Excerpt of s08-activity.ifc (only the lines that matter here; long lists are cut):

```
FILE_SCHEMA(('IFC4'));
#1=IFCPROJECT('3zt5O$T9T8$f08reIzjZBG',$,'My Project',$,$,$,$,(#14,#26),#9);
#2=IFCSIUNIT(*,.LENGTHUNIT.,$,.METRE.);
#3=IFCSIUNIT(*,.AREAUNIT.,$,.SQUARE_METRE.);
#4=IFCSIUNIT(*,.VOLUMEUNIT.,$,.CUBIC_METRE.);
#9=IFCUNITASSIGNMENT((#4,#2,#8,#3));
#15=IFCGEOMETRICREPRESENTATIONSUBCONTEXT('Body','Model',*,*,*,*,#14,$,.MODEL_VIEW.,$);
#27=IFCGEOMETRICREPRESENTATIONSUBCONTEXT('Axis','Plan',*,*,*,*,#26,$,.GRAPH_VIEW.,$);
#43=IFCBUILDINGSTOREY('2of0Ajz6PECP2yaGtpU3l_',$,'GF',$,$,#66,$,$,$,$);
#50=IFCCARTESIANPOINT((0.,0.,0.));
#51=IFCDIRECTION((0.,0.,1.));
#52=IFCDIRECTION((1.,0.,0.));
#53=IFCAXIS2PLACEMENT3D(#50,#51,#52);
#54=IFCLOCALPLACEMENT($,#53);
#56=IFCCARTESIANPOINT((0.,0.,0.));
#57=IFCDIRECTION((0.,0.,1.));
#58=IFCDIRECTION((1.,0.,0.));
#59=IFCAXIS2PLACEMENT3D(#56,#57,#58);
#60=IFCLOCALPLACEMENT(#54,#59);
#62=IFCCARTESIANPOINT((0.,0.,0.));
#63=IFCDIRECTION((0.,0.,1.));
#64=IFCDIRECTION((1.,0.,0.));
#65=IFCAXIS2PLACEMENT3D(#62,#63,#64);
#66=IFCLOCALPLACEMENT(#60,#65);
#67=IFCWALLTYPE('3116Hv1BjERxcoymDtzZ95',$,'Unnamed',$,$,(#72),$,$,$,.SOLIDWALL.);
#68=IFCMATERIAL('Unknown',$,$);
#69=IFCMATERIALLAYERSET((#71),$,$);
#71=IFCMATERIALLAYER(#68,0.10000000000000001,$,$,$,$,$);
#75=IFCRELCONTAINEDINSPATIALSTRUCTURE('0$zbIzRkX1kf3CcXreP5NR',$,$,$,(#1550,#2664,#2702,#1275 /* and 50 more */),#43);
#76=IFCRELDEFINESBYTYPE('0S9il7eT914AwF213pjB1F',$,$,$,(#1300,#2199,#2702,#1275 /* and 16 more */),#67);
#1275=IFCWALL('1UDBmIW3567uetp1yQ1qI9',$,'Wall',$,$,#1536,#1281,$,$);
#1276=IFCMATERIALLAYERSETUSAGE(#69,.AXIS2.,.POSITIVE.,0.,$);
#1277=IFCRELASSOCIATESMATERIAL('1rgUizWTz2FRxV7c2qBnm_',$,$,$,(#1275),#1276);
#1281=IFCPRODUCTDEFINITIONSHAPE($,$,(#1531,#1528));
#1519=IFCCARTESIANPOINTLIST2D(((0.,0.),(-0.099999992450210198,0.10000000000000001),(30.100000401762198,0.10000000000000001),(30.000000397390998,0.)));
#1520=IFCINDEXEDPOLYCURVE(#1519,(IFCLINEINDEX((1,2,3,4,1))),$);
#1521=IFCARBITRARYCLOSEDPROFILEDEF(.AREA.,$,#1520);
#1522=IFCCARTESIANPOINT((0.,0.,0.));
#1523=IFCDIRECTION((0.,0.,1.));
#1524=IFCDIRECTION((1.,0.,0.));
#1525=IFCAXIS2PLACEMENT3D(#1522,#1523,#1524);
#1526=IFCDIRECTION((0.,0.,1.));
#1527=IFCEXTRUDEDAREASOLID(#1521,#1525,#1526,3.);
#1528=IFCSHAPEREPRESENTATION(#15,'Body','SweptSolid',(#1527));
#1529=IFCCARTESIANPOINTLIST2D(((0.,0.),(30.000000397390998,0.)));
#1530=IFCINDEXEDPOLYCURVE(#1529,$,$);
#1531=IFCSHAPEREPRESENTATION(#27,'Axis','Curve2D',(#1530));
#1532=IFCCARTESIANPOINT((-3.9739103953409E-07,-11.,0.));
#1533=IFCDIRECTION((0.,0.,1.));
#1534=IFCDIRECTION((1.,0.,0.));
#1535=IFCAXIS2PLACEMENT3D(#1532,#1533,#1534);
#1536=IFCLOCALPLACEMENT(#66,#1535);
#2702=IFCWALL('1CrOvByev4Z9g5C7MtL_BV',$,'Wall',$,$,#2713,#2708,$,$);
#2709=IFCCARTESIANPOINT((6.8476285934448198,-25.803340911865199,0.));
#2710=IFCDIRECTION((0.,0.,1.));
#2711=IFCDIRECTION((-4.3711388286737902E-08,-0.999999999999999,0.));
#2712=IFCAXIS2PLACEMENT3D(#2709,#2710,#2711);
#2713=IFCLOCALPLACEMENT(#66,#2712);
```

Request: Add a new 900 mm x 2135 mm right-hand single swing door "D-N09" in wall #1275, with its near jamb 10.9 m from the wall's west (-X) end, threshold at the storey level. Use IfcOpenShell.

```python
import numpy as np
import ifcopenshell
import ifcopenshell.api.feature
import ifcopenshell.api.geometry
import ifcopenshell.api.root
import ifcopenshell.api.spatial
import ifcopenshell.geom
import ifcopenshell.util.element
import ifcopenshell.util.placement
import ifcopenshell.util.representation
import ifcopenshell.util.shape
import ifcopenshell.util.unit

model = ifcopenshell.open("s08-activity.ifc")
unit_scale = ifcopenshell.util.unit.calculate_unit_scale(model)
settings = ifcopenshell.geom.settings()


def volume(element):
    """Net volume in cubic metres, openings subtracted."""
    shape = ifcopenshell.geom.create_shape(settings, element)
    return ifcopenshell.util.shape.get_volume(shape.geometry)


wall = model.by_guid("1UDBmIW3567uetp1yQ1qI9")
storey = ifcopenshell.util.element.get_container(wall, ifc_class="IfcBuildingStorey")
context = ifcopenshell.util.representation.get_context(model, "Model", "Body", "MODEL_VIEW")
before = volume(wall)

width, height, from_end, sill = 0.9, 2.135, 10.9, 0.0  # metres

# The wall runs along its own X axis, and the end named is its -X end.
wall_shape = ifcopenshell.geom.create_shape(settings, wall)
x, y, z = ifcopenshell.util.shape.get_vertices(wall_shape.geometry).T
start = x.min() + from_end
face, thickness = float(y.min()), float(y.max() - y.min())
wall_matrix = ifcopenshell.util.placement.get_local_placement(wall.ObjectPlacement)
level = ifcopenshell.util.placement.get_local_placement(storey.ObjectPlacement)[2, 3]


def in_wall(x, y):
    """Placement at x, y metres in the wall's axes, at sill height."""
    matrix = wall_matrix.copy()
    matrix[:, 3] = wall_matrix @ np.array([x / unit_scale, y / unit_scale, 0.0, 1.0])
    matrix[2, 3] = level + sill / unit_scale
    return matrix


# Opening: a box that overshoots both wall faces by 50 mm.
opening = ifcopenshell.api.root.create_entity(model, ifc_class="IfcOpeningElement", predefined_type="OPENING")
box = ifcopenshell.api.geometry.add_wall_representation(
    model, context=context, length=width, height=height, thickness=thickness + 0.1
)
ifcopenshell.api.geometry.assign_representation(model, product=opening, representation=box)
ifcopenshell.api.geometry.edit_object_placement(model, product=opening, matrix=in_wall(start, face - 0.05), is_si=False)
ifcopenshell.api.feature.add_feature(model, feature=opening, element=wall)

door = ifcopenshell.api.root.create_entity(model, ifc_class="IfcDoor", name="D-N09", predefined_type="DOOR")
door.OverallWidth, door.OverallHeight = width / unit_scale, height / unit_scale
door.OperationType = "SINGLE_SWING_RIGHT"
body = ifcopenshell.api.geometry.add_door_representation(
    model,
    context=context,
    overall_width=door.OverallWidth,
    overall_height=door.OverallHeight,
    operation_type="SINGLE_SWING_RIGHT",
    lining_properties={"LiningDepth": thickness / unit_scale, "ThresholdDepth": thickness / unit_scale},
)
ifcopenshell.api.geometry.assign_representation(model, product=door, representation=body)
ifcopenshell.api.spatial.assign_container(model, products=[door], relating_structure=storey)
ifcopenshell.api.feature.add_filling(model, opening=opening, element=door)

# The lining spans the wall, so the door starts at the wall face.
ifcopenshell.api.geometry.edit_object_placement(model, product=door, matrix=in_wall(start, face), is_si=False)

after = volume(wall)

print(f"wall volume {before:.3f} -> {after:.3f} m3")

model.write("s08-activity_rev.ifc")
```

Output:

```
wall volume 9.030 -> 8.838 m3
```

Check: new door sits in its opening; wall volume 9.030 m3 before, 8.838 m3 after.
